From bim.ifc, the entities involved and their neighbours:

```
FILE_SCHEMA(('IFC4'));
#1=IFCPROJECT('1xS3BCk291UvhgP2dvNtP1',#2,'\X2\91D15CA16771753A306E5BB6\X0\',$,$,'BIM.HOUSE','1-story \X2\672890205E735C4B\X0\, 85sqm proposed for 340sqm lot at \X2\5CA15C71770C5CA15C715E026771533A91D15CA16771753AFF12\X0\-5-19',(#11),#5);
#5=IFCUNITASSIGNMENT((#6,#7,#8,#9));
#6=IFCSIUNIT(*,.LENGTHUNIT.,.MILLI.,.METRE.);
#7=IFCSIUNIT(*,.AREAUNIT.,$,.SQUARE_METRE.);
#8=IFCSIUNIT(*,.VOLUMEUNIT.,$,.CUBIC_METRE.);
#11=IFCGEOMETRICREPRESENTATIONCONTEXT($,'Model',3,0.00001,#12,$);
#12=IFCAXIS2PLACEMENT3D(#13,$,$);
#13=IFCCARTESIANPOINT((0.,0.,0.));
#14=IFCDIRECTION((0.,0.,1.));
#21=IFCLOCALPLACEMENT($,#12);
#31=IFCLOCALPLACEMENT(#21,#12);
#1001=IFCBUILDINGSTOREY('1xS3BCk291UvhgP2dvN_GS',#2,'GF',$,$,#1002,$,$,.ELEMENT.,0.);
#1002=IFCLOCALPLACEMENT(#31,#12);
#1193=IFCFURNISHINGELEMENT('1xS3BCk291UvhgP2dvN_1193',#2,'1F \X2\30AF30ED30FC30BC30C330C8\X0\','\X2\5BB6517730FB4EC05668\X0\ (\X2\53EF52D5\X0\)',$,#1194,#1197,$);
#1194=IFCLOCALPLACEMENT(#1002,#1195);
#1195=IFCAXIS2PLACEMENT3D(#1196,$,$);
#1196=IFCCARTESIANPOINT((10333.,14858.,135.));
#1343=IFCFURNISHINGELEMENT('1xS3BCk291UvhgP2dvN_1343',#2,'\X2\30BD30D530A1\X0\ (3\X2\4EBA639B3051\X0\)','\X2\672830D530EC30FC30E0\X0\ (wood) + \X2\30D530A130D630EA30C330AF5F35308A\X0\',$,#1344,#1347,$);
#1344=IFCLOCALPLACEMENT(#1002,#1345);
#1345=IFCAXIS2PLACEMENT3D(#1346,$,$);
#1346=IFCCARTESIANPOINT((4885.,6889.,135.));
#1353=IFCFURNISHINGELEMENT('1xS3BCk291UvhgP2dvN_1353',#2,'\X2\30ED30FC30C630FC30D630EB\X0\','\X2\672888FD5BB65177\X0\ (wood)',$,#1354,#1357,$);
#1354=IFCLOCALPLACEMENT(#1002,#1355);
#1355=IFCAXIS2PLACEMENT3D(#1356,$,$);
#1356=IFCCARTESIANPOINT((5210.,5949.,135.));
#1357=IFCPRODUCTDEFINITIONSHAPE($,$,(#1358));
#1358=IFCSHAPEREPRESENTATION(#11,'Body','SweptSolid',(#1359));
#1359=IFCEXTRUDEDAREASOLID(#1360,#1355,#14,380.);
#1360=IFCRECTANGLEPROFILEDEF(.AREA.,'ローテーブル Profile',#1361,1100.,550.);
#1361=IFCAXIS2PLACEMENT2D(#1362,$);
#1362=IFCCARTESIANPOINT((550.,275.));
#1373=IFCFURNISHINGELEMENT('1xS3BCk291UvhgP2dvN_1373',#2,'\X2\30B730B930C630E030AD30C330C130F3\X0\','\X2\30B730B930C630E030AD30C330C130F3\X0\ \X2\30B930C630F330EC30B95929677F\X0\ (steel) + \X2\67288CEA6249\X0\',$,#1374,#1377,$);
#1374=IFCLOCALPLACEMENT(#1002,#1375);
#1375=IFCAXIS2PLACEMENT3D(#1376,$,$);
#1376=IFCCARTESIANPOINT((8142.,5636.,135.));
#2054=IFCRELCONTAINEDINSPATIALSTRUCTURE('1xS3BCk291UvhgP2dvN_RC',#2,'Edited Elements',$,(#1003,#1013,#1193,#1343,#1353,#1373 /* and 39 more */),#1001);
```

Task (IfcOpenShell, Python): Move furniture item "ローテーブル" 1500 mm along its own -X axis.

```python
import ifcopenshell
import ifcopenshell.api.geometry
import ifcopenshell.util.placement
import ifcopenshell.util.unit

model = ifcopenshell.open("bim.ifc")
unit_scale = ifcopenshell.util.unit.calculate_unit_scale(model)

item = model.by_guid("1xS3BCk291UvhgP2dvN_1353")
matrix = ifcopenshell.util.placement.get_local_placement(item.ObjectPlacement)
matrix[:3, 3] -= matrix[:3, 0] * 1.5 / unit_scale
ifcopenshell.api.geometry.edit_object_placement(model, product=item, matrix=matrix, is_si=False)

print(ifcopenshell.util.placement.get_local_placement(item.ObjectPlacement).round(3) + 0.0)

model.write("bim_updated.ifc")
```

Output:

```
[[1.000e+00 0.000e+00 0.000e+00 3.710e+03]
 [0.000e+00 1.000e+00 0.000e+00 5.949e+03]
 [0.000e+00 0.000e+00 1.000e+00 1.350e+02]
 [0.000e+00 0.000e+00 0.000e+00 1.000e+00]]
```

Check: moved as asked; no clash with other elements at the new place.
